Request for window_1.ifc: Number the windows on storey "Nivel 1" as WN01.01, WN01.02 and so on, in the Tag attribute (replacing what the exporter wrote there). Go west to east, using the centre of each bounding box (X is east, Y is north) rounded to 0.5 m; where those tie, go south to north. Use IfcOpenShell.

First a look at what the model holds.

```python
import ifcopenshell
import ifcopenshell.util.element
import ifcopenshell.util.placement

model = ifcopenshell.open("window_1.ifc")
print(model.schema)
storey = next(s for s in model.by_type("IfcBuildingStorey") if s.Name == "Nivel 1")
windows = [e for e in ifcopenshell.util.element.get_decomposition(storey) if e.is_a("IfcWindow")]
for e in sorted(windows, key=lambda e: e.id()):
    origin = ifcopenshell.util.placement.get_local_placement(e.ObjectPlacement)[:3, 3]
    print(e.id(), e.Tag, e.Name, origin.round(2) + 0.0, sep=" | ")
```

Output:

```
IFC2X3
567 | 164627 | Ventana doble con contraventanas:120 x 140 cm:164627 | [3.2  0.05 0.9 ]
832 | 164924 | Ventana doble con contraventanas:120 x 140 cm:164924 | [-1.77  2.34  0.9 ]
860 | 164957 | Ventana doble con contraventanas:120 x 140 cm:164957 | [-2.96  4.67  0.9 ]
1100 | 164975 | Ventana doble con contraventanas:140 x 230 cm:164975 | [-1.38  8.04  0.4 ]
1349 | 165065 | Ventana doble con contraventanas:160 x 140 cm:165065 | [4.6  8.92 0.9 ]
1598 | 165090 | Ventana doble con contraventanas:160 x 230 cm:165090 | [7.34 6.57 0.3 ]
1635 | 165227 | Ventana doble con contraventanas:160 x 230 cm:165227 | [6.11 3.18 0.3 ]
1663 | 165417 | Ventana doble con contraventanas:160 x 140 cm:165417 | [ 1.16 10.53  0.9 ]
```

```python
import ifcopenshell
import ifcopenshell.geom
import ifcopenshell.util.element
import ifcopenshell.util.shape

model = ifcopenshell.open("window_1.ifc")
settings = ifcopenshell.geom.settings()
settings.set("use-world-coords", True)


def centre(element):
    shape = ifcopenshell.geom.create_shape(settings, element)
    return ifcopenshell.util.shape.get_bbox_centroid(shape.geometry)


storey = next(s for s in model.by_type("IfcBuildingStorey") if s.Name == "Nivel 1")
windows = [e for e in ifcopenshell.util.element.get_decomposition(storey) if e.is_a("IfcWindow")]

# Insertion points can sit at a corner or the storey origin, so sort by the geometry (in metres).
centres = {e: centre(e) for e in windows}
windows.sort(key=lambda e: (round(centres[e][0] / 0.5), centres[e][1]))

for i, e in enumerate(windows, start=1):
    number = f"WN01.{i:02d}"
    e.Tag = number
    print(e.id(), number)

model.write("window_1_rev.ifc")
```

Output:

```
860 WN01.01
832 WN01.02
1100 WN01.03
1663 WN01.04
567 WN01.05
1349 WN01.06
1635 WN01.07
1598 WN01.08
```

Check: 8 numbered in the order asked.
